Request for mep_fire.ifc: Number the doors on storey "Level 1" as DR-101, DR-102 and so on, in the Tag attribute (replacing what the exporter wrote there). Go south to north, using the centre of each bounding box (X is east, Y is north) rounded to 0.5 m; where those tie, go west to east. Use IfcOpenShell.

First a look at what the model holds.

```python
import ifcopenshell
import ifcopenshell.util.element
import ifcopenshell.util.placement

model = ifcopenshell.open("mep_fire.ifc")
print(model.schema)
storey = next(s for s in model.by_type("IfcBuildingStorey") if s.Name == "Level 1")
doors = [e for e in ifcopenshell.util.element.get_decomposition(storey) if e.is_a("IfcDoor")]
for e in sorted(doors, key=lambda e: e.id()):
    origin = ifcopenshell.util.placement.get_local_placement(e.ObjectPlacement)[:3, 3]
    print(e.id(), e.Tag, e.Name, origin.round(2) + 0.0, sep=" | ")
```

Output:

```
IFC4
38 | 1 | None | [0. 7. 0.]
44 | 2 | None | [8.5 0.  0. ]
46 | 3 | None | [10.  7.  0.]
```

```python
import ifcopenshell
import ifcopenshell.geom
import ifcopenshell.util.element
import ifcopenshell.util.shape

model = ifcopenshell.open("mep_fire.ifc")
settings = ifcopenshell.geom.settings()
settings.set("use-world-coords", True)


def centre(element):
    shape = ifcopenshell.geom.create_shape(settings, element)
    return ifcopenshell.util.shape.get_bbox_centroid(shape.geometry)


storey = next(s for s in model.by_type("IfcBuildingStorey") if s.Name == "Level 1")
doors = [e for e in ifcopenshell.util.element.get_decomposition(storey) if e.is_a("IfcDoor")]

# Insertion points can sit at a corner or the storey origin, so sort by the geometry (in metres).
centres = {e: centre(e) for e in doors}
doors.sort(key=lambda e: (round(centres[e][1] / 0.5), centres[e][0]))

for i, e in enumerate(doors, start=1):
    number = f"DR-1{i:02d}"
    e.Tag = number
    print(e.id(), number)

model.write("mep_fire_v2.ifc")
```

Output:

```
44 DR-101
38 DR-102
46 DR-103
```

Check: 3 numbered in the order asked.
